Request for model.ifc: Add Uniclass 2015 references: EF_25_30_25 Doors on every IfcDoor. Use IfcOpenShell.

First a look at what the model holds.

```python
import ifcopenshell

model = ifcopenshell.open("model.ifc")
print(model.schema)
print("classifications:", [c.Name for c in model.by_type("IfcClassification")])
for ifc_class in ("IfcDoor", "IfcRoof", "IfcStair", "IfcWall", "IfcWindow"):
    print(ifc_class, len(model.by_type(ifc_class)))
```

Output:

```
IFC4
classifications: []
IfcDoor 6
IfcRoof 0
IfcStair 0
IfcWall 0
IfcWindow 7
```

```python
import ifcopenshell
import ifcopenshell.api.classification

model = ifcopenshell.open("model.ifc")

system = ifcopenshell.api.classification.add_classification(model, classification="Uniclass 2015")

codes = {
    "IfcDoor": ("EF_25_30_25", "Doors"),
}
for ifc_class, (code, name) in codes.items():
    products = model.by_type(ifc_class)
    ifcopenshell.api.classification.add_reference(
        model, products=products, classification=system, identification=code, name=name
    )
    print(code, len(products))

model.write("model_updated.ifc")
```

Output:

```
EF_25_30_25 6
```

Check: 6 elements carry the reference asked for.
